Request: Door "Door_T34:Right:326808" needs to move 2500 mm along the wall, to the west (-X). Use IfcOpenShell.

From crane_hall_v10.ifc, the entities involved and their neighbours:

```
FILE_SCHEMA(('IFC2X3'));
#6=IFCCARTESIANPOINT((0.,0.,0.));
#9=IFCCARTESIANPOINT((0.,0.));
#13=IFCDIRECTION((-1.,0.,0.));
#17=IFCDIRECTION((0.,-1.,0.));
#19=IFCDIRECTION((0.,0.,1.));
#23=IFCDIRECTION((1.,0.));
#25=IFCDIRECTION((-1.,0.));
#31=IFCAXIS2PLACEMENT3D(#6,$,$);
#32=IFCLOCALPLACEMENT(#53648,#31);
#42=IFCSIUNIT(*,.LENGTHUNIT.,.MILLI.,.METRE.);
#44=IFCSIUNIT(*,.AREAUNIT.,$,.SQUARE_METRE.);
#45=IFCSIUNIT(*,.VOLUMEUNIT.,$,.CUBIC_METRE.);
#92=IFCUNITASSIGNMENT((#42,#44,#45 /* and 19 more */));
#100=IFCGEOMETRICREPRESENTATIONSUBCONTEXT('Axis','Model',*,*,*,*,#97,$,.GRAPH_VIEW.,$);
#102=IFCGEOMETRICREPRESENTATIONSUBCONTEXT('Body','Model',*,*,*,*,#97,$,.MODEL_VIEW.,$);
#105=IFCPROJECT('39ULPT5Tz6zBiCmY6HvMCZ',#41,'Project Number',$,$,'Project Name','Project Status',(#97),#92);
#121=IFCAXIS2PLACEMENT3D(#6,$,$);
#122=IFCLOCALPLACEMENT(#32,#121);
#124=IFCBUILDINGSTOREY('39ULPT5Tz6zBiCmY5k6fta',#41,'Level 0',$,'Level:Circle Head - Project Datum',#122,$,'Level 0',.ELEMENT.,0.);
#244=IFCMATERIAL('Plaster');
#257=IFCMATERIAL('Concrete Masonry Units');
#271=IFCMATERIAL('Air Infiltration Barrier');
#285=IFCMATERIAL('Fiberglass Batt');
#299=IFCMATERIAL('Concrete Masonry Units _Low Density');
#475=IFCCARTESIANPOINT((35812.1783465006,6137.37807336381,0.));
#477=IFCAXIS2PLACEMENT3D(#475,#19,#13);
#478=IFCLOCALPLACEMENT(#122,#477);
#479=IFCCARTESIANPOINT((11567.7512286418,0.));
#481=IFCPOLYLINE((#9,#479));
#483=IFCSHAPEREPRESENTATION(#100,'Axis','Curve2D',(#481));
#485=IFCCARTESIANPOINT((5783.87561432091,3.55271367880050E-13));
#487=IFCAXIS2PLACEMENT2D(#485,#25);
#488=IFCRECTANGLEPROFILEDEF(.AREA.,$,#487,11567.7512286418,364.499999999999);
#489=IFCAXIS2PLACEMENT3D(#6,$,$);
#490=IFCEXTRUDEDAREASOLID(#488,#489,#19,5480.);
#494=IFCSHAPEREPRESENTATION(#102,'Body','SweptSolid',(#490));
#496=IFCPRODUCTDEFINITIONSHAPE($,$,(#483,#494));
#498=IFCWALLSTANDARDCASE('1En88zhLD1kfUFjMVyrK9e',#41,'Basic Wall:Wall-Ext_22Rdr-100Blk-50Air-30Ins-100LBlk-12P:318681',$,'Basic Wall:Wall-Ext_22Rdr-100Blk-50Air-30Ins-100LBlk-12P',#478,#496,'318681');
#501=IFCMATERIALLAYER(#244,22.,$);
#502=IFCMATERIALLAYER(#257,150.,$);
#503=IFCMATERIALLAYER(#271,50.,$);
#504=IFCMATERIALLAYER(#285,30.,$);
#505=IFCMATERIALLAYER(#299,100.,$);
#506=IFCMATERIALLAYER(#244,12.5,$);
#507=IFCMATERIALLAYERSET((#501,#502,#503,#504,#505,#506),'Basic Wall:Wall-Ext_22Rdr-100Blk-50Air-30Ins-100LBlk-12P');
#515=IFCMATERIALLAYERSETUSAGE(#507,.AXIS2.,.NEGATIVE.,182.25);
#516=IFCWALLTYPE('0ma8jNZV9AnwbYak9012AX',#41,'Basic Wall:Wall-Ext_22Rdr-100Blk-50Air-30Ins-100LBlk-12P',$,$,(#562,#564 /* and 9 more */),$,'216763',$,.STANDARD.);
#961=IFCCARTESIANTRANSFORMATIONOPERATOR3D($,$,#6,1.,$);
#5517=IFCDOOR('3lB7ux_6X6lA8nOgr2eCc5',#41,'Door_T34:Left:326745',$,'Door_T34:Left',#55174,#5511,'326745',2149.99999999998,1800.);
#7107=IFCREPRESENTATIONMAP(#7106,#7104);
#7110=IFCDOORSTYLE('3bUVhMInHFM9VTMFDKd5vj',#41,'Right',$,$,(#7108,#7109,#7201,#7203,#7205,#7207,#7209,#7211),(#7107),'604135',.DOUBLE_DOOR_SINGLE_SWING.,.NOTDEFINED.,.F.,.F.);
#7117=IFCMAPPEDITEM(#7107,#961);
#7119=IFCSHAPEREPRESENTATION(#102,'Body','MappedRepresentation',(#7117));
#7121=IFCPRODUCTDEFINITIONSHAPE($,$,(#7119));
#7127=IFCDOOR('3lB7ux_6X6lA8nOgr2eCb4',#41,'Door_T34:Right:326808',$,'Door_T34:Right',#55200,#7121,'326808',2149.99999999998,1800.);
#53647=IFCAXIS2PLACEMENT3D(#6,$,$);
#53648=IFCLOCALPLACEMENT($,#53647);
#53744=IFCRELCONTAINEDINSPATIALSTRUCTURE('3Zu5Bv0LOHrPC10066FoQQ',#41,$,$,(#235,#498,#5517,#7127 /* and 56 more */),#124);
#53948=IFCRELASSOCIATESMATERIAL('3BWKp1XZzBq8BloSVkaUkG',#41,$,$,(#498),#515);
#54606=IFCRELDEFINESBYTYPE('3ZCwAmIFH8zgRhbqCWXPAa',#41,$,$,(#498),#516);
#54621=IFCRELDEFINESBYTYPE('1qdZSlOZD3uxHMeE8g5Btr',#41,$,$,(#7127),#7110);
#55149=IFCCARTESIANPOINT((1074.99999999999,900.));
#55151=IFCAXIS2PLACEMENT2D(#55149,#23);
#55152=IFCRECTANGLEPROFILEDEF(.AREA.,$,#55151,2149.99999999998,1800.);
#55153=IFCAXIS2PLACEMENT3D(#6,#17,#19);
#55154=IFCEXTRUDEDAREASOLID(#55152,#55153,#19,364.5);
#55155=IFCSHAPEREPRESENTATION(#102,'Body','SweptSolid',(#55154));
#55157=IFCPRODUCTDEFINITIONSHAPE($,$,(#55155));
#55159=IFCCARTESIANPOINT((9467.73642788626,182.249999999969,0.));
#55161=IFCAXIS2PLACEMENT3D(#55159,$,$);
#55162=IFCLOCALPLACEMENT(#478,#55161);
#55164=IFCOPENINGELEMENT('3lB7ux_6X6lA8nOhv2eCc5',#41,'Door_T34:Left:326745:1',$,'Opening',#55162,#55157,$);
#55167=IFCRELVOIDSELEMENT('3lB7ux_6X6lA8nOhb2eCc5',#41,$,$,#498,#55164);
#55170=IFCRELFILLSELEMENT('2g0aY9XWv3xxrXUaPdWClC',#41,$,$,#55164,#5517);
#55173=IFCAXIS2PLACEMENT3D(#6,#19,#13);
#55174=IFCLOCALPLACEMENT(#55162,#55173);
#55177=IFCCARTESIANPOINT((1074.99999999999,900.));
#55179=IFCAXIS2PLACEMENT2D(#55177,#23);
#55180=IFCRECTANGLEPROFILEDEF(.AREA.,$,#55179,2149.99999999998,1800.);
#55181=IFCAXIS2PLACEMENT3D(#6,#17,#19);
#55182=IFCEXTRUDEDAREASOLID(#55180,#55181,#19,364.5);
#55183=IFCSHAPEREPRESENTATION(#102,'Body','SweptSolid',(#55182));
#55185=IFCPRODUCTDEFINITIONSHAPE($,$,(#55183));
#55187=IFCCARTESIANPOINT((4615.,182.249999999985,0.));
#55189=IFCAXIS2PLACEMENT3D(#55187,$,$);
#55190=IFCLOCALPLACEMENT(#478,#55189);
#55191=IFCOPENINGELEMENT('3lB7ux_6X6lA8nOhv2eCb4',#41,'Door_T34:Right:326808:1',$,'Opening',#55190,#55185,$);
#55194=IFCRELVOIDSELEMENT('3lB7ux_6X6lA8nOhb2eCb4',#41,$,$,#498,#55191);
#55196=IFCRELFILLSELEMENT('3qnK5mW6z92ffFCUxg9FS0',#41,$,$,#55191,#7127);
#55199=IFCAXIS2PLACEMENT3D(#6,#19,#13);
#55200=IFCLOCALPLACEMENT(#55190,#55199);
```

```python
import ifcopenshell
import ifcopenshell.api.geometry
import ifcopenshell.util.placement

model = ifcopenshell.open("crane_hall_v10.ifc")

door = model.by_guid("3lB7ux_6X6lA8nOgr2eCb4")
opening = door.FillsVoids[0].RelatingOpeningElement
wall = opening.VoidsElements[0].RelatingBuildingElement

wall_matrix = ifcopenshell.util.placement.get_local_placement(wall.ObjectPlacement)
shift = wall_matrix[:3, 0] * 2500.0
before = ifcopenshell.util.placement.get_local_placement(door.ObjectPlacement)[:3, 3].copy()

# The door is placed relative to its opening, so it follows when the opening moves.
matrix = ifcopenshell.util.placement.get_local_placement(opening.ObjectPlacement)
matrix[:3, 3] += shift
ifcopenshell.api.geometry.edit_object_placement(
    model, product=opening, matrix=matrix, is_si=False, should_transform_children=True
)

after = ifcopenshell.util.placement.get_local_placement(door.ObjectPlacement)[:3, 3]
print("door moved by", (after - before).round(3) + 0.0)

model.write("crane_hall_v10_edited.ifc")
```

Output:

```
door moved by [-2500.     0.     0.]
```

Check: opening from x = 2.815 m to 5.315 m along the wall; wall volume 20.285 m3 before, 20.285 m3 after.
